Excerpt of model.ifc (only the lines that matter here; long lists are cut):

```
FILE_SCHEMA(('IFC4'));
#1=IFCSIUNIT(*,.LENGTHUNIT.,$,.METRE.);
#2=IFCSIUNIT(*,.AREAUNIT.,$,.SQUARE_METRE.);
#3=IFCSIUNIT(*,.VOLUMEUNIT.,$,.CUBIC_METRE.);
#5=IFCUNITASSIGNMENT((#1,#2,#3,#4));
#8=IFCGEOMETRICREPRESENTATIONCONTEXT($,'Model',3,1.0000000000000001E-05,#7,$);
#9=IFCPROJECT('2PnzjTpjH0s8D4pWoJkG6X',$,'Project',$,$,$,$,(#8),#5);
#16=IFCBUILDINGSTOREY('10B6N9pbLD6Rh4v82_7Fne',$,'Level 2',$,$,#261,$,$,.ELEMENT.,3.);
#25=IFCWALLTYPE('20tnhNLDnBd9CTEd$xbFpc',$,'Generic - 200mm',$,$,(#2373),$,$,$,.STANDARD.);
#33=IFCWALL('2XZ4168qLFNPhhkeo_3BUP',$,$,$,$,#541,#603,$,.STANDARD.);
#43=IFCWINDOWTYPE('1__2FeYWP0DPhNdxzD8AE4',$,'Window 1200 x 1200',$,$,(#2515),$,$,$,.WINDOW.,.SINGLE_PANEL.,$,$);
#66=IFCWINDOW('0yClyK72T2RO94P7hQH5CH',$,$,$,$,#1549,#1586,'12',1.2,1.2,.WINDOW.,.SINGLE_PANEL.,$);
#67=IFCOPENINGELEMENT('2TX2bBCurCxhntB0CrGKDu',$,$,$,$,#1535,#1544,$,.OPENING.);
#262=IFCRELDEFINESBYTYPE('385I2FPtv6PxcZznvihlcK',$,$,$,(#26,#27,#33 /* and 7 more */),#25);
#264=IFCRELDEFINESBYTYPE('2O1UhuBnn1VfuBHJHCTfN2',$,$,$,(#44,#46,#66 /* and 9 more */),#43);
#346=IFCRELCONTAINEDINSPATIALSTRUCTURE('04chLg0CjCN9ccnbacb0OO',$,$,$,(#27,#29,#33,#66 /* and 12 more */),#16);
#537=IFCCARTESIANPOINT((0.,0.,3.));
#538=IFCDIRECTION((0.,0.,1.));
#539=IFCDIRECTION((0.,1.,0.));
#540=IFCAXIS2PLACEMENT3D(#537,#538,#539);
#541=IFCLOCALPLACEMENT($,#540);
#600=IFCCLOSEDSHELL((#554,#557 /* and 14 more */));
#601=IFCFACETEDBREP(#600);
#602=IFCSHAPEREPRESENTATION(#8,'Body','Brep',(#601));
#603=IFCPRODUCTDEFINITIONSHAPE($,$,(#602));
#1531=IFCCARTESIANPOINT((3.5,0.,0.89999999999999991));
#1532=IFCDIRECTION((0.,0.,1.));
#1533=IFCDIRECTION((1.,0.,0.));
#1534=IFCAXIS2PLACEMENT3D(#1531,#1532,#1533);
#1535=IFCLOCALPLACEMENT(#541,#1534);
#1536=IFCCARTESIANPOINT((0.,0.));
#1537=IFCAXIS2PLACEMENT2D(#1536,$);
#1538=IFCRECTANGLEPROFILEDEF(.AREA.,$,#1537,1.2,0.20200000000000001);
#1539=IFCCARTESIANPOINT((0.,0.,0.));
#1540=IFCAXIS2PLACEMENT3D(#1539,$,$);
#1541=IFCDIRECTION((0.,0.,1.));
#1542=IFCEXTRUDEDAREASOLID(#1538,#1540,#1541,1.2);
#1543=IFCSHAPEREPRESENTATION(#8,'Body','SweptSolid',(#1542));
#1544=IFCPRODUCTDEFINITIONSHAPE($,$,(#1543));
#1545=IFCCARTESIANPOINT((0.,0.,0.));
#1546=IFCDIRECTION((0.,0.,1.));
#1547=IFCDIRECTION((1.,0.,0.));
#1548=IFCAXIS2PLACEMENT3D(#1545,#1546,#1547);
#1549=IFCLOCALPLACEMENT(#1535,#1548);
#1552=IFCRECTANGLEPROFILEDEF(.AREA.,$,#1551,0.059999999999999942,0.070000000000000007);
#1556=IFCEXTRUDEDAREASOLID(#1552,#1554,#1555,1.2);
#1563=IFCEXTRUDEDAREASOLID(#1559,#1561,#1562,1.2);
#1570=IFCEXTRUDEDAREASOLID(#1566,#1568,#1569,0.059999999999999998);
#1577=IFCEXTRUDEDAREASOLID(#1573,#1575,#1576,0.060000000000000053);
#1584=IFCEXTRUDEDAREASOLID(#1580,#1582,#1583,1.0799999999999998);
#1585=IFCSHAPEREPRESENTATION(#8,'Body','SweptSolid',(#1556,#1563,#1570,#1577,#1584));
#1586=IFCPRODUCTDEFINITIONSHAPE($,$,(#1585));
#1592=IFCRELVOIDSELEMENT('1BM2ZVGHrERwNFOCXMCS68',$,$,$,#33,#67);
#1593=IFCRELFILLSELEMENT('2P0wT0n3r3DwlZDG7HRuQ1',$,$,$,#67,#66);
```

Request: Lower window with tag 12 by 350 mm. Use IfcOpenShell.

```python
import numpy as np
import ifcopenshell
import ifcopenshell.api.geometry
import ifcopenshell.util.placement
import ifcopenshell.util.unit

model = ifcopenshell.open("model.ifc")
unit_scale = ifcopenshell.util.unit.calculate_unit_scale(model)

window = model.by_guid("0yClyK72T2RO94P7hQH5CH")
opening = window.FillsVoids[0].RelatingOpeningElement
dz = -0.35 / unit_scale

shift = np.array([0.0, 0.0, dz])
# The window is placed relative to its opening, so it follows when the opening moves.
matrix = ifcopenshell.util.placement.get_local_placement(opening.ObjectPlacement)
matrix[:3, 3] += shift
ifcopenshell.api.geometry.edit_object_placement(
    model, product=opening, matrix=matrix, is_si=False, should_transform_children=True
)

print(f"moved by {dz * unit_scale:+.3f} m")

model.write("model-out.ifc")
```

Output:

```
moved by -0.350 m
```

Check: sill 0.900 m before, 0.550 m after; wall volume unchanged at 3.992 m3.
